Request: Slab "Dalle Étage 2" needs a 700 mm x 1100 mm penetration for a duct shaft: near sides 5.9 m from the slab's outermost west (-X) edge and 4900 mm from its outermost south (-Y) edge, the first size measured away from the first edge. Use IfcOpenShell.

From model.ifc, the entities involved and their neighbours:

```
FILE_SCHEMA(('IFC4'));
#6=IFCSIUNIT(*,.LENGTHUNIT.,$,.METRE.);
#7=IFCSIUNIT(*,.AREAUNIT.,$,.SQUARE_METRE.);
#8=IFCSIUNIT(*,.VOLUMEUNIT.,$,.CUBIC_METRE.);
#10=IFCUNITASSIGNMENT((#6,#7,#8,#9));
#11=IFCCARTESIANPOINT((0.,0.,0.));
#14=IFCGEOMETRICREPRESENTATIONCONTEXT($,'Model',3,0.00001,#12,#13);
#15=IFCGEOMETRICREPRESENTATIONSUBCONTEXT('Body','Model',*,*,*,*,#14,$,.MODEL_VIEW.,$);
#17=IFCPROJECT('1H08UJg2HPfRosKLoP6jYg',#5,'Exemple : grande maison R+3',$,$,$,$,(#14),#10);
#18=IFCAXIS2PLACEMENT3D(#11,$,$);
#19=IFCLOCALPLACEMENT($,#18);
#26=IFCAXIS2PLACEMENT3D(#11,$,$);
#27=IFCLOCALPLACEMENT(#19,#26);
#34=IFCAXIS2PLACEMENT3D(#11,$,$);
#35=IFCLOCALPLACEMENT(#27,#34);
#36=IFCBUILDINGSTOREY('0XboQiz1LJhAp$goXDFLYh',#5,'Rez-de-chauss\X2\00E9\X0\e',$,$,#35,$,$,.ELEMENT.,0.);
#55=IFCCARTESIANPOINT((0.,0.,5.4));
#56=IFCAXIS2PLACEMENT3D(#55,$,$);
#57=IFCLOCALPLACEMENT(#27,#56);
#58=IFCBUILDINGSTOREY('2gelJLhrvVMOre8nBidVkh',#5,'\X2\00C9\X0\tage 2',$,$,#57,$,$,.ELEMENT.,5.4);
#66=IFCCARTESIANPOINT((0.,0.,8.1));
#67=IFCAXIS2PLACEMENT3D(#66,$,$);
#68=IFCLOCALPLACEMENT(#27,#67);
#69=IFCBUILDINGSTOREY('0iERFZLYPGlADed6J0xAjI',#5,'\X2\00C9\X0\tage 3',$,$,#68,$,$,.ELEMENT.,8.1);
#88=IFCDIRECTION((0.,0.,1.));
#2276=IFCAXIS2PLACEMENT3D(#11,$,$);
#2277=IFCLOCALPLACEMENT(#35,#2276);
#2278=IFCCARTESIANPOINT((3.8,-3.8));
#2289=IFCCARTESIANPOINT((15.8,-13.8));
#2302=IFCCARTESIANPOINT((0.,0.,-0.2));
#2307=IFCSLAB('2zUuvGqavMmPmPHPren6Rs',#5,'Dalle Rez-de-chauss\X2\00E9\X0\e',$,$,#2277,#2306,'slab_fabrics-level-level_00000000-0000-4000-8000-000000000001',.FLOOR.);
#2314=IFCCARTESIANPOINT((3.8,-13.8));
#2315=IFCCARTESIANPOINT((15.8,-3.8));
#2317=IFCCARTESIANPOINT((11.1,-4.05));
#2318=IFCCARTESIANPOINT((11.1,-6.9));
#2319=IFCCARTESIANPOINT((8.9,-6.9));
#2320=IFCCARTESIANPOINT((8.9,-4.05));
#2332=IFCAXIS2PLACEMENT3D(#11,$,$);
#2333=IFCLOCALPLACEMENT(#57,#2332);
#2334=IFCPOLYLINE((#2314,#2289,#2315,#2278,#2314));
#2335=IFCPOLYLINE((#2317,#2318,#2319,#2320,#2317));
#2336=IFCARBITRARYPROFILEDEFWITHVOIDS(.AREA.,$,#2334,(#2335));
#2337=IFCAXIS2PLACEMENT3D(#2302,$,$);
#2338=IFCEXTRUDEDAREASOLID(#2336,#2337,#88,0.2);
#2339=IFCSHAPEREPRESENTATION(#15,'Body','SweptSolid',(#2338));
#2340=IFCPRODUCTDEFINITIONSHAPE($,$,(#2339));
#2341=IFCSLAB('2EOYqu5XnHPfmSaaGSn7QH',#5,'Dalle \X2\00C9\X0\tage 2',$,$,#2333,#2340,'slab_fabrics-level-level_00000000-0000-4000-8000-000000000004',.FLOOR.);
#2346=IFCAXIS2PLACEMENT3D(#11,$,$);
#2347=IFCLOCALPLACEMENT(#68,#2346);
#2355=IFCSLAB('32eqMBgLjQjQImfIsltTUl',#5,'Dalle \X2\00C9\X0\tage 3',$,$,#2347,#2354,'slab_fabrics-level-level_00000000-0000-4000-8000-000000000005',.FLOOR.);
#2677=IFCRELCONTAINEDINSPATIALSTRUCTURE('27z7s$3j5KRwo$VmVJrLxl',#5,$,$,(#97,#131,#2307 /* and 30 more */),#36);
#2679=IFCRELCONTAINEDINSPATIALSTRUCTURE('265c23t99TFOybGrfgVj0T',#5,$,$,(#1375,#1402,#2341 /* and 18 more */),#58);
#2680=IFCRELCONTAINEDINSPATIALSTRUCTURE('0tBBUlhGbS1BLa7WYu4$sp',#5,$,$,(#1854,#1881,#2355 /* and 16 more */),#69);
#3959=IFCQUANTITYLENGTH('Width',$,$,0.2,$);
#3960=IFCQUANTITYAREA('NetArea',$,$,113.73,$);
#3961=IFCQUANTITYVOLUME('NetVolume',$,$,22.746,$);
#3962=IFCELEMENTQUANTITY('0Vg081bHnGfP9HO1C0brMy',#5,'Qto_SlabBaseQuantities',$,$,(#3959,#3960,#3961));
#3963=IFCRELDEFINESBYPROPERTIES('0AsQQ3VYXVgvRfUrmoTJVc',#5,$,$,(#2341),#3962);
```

```python
import numpy as np
import ifcopenshell
import ifcopenshell.api.feature
import ifcopenshell.api.geometry
import ifcopenshell.api.pset
import ifcopenshell.api.root
import ifcopenshell.geom
import ifcopenshell.util.element
import ifcopenshell.util.placement
import ifcopenshell.util.representation
import ifcopenshell.util.shape
import ifcopenshell.util.unit

model = ifcopenshell.open("model.ifc")
unit_scale = ifcopenshell.util.unit.calculate_unit_scale(model)
area_scale = ifcopenshell.util.unit.calculate_unit_scale(model, "AREAUNIT")
volume_scale = ifcopenshell.util.unit.calculate_unit_scale(model, "VOLUMEUNIT")
settings = ifcopenshell.geom.settings()


def volume(element):
    """Net volume in cubic metres, openings subtracted."""
    shape = ifcopenshell.geom.create_shape(settings, element)
    return ifcopenshell.util.shape.get_volume(shape.geometry)


slab = model.by_id(2341)
before = volume(slab)

# Extent in the slab's own axes, in metres. The edges named are its -X and -Y sides.
slab_shape = ifcopenshell.geom.create_shape(settings, slab)
vertices = ifcopenshell.util.shape.get_vertices(slab_shape.geometry)
x_min, y_min, bottom = vertices.min(axis=0)
top = vertices[:, 2].max()

opening = ifcopenshell.api.root.create_entity(model, ifc_class="IfcOpeningElement", name="Duct shaft opening", predefined_type="OPENING")
context = ifcopenshell.util.representation.get_context(model, "Model", "Body", "MODEL_VIEW")
width, depth = 0.7, 1.1
outline = [(0.0, 0.0), (width, 0.0), (width, depth), (0.0, depth), (0.0, 0.0)]
# Overshoot both faces by 50 mm so the cut is clean.
shape = ifcopenshell.api.geometry.add_slab_representation(
    model, context=context, depth=top - bottom + 0.1, polyline=outline
)
ifcopenshell.api.geometry.assign_representation(model, product=opening, representation=shape)

matrix = ifcopenshell.util.placement.get_local_placement(slab.ObjectPlacement)
matrix[:, 3] = matrix @ np.append(np.array([x_min + 5.9, y_min + 4.9, bottom - 0.05]) / unit_scale, 1.0)
ifcopenshell.api.geometry.edit_object_placement(model, product=opening, matrix=matrix, is_si=False)
ifcopenshell.api.feature.add_feature(model, feature=opening, element=slab)

after = volume(slab)

# Update the slab's stored quantities.
qto = model.by_id(ifcopenshell.util.element.get_pset(slab, "Qto_SlabBaseQuantities", should_inherit=False)["id"])
ifcopenshell.api.pset.edit_qto(model, qto=qto, properties={
    "NetArea": after / (top - bottom) / area_scale,
    "NetVolume": after / volume_scale,
})

print(f"slab volume {before:.3f} -> {after:.3f} m3")

model.write("model_v2.ifc")
```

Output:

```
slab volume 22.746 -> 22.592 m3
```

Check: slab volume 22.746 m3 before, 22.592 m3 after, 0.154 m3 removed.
